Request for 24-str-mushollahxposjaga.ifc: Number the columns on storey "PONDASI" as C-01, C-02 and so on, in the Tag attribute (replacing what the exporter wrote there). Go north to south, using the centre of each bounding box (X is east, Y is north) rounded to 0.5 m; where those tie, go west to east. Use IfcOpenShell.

First a look at what the model holds.

```python
import ifcopenshell
import ifcopenshell.util.element
import ifcopenshell.util.placement

model = ifcopenshell.open("24-str-mushollahxposjaga.ifc")
print(model.schema)
storey = next(s for s in model.by_type("IfcBuildingStorey") if s.Name == "PONDASI")
columns = [e for e in ifcopenshell.util.element.get_decomposition(storey) if e.is_a("IfcColumn")]
for e in sorted(columns, key=lambda e: e.id()):
    origin = ifcopenshell.util.placement.get_local_placement(e.ObjectPlacement)[:3, 3]
    print(e.id(), e.Tag, e.Name, origin.round(2) + 0.0, sep=" | ")
```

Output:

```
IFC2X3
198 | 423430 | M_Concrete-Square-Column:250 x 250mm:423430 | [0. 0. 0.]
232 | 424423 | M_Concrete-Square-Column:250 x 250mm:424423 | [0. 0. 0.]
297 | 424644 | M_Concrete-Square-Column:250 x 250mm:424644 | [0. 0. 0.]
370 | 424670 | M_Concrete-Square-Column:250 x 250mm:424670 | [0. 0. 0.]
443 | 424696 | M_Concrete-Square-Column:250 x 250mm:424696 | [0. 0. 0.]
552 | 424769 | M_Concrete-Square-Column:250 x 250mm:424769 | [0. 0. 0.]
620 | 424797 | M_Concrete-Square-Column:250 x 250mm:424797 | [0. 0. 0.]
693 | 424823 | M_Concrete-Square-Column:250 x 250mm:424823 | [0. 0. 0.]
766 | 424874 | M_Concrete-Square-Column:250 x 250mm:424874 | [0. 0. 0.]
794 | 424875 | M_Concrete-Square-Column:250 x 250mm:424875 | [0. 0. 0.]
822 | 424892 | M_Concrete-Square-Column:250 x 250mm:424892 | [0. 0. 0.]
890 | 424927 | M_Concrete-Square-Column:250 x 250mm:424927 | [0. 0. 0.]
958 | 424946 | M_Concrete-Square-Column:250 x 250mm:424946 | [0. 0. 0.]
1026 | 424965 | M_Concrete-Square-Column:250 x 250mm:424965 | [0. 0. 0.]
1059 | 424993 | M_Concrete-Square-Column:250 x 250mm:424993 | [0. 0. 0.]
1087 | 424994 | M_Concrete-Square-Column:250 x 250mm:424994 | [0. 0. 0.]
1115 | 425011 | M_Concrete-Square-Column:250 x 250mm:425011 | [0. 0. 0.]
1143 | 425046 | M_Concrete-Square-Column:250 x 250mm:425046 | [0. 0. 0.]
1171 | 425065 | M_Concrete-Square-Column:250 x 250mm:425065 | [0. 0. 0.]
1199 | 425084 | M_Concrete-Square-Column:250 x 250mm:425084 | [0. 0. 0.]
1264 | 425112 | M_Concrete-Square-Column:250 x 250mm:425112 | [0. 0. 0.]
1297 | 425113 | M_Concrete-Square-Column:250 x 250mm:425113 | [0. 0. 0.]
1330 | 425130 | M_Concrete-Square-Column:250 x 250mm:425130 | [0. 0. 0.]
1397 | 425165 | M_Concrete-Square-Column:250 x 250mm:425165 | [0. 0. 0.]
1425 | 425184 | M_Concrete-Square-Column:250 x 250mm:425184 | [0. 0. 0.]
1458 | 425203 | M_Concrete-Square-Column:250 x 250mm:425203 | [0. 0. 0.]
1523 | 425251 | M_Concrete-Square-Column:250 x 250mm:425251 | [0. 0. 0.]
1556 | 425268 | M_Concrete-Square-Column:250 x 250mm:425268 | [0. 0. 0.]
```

```python
import ifcopenshell
import ifcopenshell.geom
import ifcopenshell.util.element
import ifcopenshell.util.shape

model = ifcopenshell.open("24-str-mushollahxposjaga.ifc")
settings = ifcopenshell.geom.settings()
settings.set("use-world-coords", True)


def centre(element):
    shape = ifcopenshell.geom.create_shape(settings, element)
    return ifcopenshell.util.shape.get_bbox_centroid(shape.geometry)


storey = next(s for s in model.by_type("IfcBuildingStorey") if s.Name == "PONDASI")
columns = [e for e in ifcopenshell.util.element.get_decomposition(storey) if e.is_a("IfcColumn")]

# Insertion points can sit at a corner or the storey origin, so sort by the geometry (in metres).
centres = {e: centre(e) for e in columns}
columns.sort(key=lambda e: (-round(centres[e][1] / 0.5), centres[e][0]))

for i, e in enumerate(columns, start=1):
    number = f"C-{i:02d}"
    e.Tag = number
    print(e.id(), number)

model.write("24-str-mushollahxposjaga_v2.ifc")
```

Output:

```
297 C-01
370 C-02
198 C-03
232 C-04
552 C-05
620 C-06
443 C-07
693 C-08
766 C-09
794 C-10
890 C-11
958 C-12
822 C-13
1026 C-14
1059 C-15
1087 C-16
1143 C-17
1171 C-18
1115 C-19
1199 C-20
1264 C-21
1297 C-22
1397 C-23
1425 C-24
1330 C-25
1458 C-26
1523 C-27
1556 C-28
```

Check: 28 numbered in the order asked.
